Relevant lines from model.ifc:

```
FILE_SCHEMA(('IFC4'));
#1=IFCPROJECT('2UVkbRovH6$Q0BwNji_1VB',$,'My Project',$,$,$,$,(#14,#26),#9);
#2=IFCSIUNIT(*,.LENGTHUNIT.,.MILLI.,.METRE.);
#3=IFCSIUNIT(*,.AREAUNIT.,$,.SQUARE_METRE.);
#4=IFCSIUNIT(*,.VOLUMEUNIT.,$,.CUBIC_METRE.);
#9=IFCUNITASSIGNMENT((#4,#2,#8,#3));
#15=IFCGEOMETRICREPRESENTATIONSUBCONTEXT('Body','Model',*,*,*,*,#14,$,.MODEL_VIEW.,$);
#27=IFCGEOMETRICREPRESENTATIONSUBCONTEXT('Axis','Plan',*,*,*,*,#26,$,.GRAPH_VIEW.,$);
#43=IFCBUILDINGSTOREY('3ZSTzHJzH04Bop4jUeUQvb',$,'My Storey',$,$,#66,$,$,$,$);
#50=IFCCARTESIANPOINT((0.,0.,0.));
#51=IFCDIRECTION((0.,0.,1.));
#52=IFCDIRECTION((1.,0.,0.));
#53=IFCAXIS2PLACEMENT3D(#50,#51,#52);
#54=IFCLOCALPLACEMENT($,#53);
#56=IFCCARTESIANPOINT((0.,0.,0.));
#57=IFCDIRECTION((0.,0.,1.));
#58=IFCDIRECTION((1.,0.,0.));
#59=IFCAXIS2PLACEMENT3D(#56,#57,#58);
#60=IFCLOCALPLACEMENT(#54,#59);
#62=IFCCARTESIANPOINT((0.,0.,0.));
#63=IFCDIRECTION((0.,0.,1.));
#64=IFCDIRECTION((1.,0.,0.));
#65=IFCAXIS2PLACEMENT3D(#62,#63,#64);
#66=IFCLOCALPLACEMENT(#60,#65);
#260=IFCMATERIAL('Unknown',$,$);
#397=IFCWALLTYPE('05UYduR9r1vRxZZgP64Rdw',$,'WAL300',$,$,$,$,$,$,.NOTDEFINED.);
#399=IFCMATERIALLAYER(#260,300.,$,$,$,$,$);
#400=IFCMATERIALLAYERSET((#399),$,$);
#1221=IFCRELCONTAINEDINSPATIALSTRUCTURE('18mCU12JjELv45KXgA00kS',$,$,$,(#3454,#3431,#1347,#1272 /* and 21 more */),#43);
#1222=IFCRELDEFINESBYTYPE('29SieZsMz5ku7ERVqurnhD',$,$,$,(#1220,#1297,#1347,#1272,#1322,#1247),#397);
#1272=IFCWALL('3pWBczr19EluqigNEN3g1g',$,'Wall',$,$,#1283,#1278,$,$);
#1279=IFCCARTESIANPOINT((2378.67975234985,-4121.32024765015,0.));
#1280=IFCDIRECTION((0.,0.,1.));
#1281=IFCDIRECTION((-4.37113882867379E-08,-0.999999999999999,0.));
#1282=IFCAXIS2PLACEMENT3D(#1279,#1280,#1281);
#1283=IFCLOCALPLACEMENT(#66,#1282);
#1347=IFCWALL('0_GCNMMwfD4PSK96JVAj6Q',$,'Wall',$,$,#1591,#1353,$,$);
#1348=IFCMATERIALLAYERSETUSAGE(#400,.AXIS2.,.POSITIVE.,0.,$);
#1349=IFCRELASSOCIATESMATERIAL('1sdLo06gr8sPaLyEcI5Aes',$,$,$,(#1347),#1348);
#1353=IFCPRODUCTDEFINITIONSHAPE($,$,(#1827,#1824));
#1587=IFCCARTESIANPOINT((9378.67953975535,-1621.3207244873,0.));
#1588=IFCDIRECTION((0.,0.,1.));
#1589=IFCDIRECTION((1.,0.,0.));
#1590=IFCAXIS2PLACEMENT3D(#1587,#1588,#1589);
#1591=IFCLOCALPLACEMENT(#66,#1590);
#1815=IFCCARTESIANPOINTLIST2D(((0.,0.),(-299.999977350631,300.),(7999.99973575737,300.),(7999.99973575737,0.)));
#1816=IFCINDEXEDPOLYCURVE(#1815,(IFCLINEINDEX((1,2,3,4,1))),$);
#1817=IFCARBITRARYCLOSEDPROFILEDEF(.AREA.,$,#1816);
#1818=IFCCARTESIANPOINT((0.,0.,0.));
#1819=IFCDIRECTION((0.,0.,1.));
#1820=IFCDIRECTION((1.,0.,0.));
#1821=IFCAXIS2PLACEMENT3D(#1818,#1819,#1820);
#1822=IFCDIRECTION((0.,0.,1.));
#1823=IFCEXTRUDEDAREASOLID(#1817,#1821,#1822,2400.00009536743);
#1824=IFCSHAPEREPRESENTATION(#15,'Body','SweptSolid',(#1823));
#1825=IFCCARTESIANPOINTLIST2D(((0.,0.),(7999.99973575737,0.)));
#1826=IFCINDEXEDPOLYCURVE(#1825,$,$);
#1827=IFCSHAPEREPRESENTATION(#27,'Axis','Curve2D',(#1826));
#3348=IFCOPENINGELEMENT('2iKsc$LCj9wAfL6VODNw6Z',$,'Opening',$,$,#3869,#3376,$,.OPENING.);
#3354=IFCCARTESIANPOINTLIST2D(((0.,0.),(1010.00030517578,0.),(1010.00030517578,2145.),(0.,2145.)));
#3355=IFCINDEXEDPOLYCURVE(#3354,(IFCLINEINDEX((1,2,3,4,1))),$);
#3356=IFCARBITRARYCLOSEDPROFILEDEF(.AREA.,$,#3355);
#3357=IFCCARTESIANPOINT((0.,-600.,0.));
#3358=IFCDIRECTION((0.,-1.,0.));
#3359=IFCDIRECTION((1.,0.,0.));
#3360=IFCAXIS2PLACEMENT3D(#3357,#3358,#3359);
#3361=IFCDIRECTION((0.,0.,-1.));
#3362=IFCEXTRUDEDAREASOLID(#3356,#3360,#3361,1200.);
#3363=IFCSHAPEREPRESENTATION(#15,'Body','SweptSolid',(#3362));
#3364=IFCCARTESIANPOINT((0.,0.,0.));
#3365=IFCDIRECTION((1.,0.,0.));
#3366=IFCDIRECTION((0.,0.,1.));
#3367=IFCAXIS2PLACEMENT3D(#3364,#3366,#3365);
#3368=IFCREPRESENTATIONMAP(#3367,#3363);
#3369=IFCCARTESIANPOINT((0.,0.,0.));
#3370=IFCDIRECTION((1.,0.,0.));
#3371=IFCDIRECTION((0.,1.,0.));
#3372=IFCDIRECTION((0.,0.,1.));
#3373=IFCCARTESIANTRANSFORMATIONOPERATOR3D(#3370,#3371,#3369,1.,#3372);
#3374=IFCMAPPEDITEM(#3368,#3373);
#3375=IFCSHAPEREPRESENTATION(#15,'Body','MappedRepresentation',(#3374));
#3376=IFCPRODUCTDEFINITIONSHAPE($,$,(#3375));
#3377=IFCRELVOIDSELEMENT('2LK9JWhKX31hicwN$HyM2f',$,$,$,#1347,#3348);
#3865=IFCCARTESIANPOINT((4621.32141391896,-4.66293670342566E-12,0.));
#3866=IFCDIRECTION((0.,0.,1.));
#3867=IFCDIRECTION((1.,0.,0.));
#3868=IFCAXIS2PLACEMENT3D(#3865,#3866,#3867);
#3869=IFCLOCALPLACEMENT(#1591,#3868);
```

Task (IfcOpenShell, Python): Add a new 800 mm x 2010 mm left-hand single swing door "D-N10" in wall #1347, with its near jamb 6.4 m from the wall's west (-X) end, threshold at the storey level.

```python
import numpy as np
import ifcopenshell
import ifcopenshell.api.feature
import ifcopenshell.api.geometry
import ifcopenshell.api.root
import ifcopenshell.api.spatial
import ifcopenshell.geom
import ifcopenshell.util.element
import ifcopenshell.util.placement
import ifcopenshell.util.representation
import ifcopenshell.util.shape
import ifcopenshell.util.unit

model = ifcopenshell.open("model.ifc")
unit_scale = ifcopenshell.util.unit.calculate_unit_scale(model)
settings = ifcopenshell.geom.settings()


def volume(element):
    """Net volume in cubic metres, openings subtracted."""
    shape = ifcopenshell.geom.create_shape(settings, element)
    return ifcopenshell.util.shape.get_volume(shape.geometry)


wall = model.by_guid("0_GCNMMwfD4PSK96JVAj6Q")
storey = ifcopenshell.util.element.get_container(wall, ifc_class="IfcBuildingStorey")
context = ifcopenshell.util.representation.get_context(model, "Model", "Body", "MODEL_VIEW")
before = volume(wall)

width, height, from_end, sill = 0.8, 2.01, 6.4, 0.0  # metres

# The wall runs along its own X axis, and the end named is its -X end.
wall_shape = ifcopenshell.geom.create_shape(settings, wall)
x, y, z = ifcopenshell.util.shape.get_vertices(wall_shape.geometry).T
start = x.min() + from_end
face, thickness = float(y.min()), float(y.max() - y.min())
wall_matrix = ifcopenshell.util.placement.get_local_placement(wall.ObjectPlacement)
level = ifcopenshell.util.placement.get_local_placement(storey.ObjectPlacement)[2, 3]


def in_wall(x, y):
    """Placement at x, y metres in the wall's axes, at sill height."""
    matrix = wall_matrix.copy()
    matrix[:, 3] = wall_matrix @ np.array([x / unit_scale, y / unit_scale, 0.0, 1.0])
    matrix[2, 3] = level + sill / unit_scale
    return matrix


# Opening: a box that overshoots both wall faces by 50 mm.
opening = ifcopenshell.api.root.create_entity(model, ifc_class="IfcOpeningElement", predefined_type="OPENING")
box = ifcopenshell.api.geometry.add_wall_representation(
    model, context=context, length=width, height=height, thickness=thickness + 0.1
)
ifcopenshell.api.geometry.assign_representation(model, product=opening, representation=box)
ifcopenshell.api.geometry.edit_object_placement(model, product=opening, matrix=in_wall(start, face - 0.05), is_si=False)
ifcopenshell.api.feature.add_feature(model, feature=opening, element=wall)

door = ifcopenshell.api.root.create_entity(model, ifc_class="IfcDoor", name="D-N10", predefined_type="DOOR")
door.OverallWidth, door.OverallHeight = width / unit_scale, height / unit_scale
door.OperationType = "SINGLE_SWING_LEFT"
body = ifcopenshell.api.geometry.add_door_representation(
    model,
    context=context,
    overall_width=door.OverallWidth,
    overall_height=door.OverallHeight,
    operation_type="SINGLE_SWING_LEFT",
    lining_properties={"LiningDepth": thickness / unit_scale, "ThresholdDepth": thickness / unit_scale},
)
ifcopenshell.api.geometry.assign_representation(model, product=door, representation=body)
ifcopenshell.api.spatial.assign_container(model, products=[door], relating_structure=storey)
ifcopenshell.api.feature.add_filling(model, opening=opening, element=door)

# The lining spans the wall, so the door starts at the wall face.
ifcopenshell.api.geometry.edit_object_placement(model, product=door, matrix=in_wall(start, face), is_si=False)

after = volume(wall)

print(f"wall volume {before:.3f} -> {after:.3f} m3")

model.write("model_rev.ifc")
```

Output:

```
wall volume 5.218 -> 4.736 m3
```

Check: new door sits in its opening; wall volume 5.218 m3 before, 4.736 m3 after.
